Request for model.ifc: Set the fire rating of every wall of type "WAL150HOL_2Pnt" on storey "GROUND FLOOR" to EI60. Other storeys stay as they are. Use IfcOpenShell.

First a look at what the model holds.

```python
import ifcopenshell
import ifcopenshell.util.element

model = ifcopenshell.open("model.ifc")
print(model.schema)
storey = next(s for s in model.by_type("IfcBuildingStorey") if s.Name == "GROUND FLOOR")
walls = [e for e in ifcopenshell.util.element.get_decomposition(storey) if e.is_a("IfcWall")]
seen = {}
for e in walls:
    element_type = ifcopenshell.util.element.get_type(e)
    key = (element_type.Name if element_type != e and element_type else None, ifcopenshell.util.element.get_pset(e, "Pset_WallCommon", "FireRating"))
    seen[key] = seen.get(key, 0) + 1
for (name, value), count in sorted(seen.items(), key=str):
    print(count, "x", name, "|", value)
```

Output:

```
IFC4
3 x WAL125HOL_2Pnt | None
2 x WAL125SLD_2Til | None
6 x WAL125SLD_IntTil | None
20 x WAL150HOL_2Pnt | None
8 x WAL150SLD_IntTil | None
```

```python
import ifcopenshell
import ifcopenshell.api.pset
import ifcopenshell.util.element

model = ifcopenshell.open("model.ifc")

storey = next(s for s in model.by_type("IfcBuildingStorey") if s.Name == "GROUND FLOOR")
walls = [e for e in ifcopenshell.util.element.get_decomposition(storey) if e.is_a("IfcWall")]

count = 0
for e in walls:
    element_type = ifcopenshell.util.element.get_type(e)
    if element_type in (None, e) or element_type.Name != "WAL150HOL_2Pnt":
        continue
    # add_pset returns the element's existing set when there is one.
    pset = ifcopenshell.api.pset.add_pset(model, product=e, name="Pset_WallCommon")
    ifcopenshell.api.pset.edit_pset(model, pset=pset, properties={"FireRating": "EI60"})
    count += 1

print(count, "walls updated")

model.write("model_rev.ifc")
```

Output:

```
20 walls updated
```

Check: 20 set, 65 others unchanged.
